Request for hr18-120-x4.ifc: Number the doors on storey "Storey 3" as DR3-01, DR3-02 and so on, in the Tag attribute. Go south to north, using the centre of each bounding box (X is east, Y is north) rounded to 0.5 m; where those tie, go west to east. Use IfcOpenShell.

First a look at what the model holds.

```python
import ifcopenshell
import ifcopenshell.util.element
import ifcopenshell.util.placement

model = ifcopenshell.open("hr18-120-x4.ifc")
print(model.schema)
storey = next(s for s in model.by_type("IfcBuildingStorey") if s.Name == "Storey 3")
doors = [e for e in ifcopenshell.util.element.get_decomposition(storey) if e.is_a("IfcDoor")]
for e in sorted(doors, key=lambda e: e.id()):
    origin = ifcopenshell.util.placement.get_local_placement(e.ObjectPlacement)[:3, 3]
    print(e.id(), e.Tag, e.Name, origin.round(2) + 0.0, sep=" | ")
```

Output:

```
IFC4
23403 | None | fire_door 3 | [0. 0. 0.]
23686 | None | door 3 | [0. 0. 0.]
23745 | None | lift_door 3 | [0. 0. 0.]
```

```python
import ifcopenshell
import ifcopenshell.geom
import ifcopenshell.util.element
import ifcopenshell.util.shape

model = ifcopenshell.open("hr18-120-x4.ifc")
settings = ifcopenshell.geom.settings()
settings.set("use-world-coords", True)


def centre(element):
    shape = ifcopenshell.geom.create_shape(settings, element)
    return ifcopenshell.util.shape.get_bbox_centroid(shape.geometry)


storey = next(s for s in model.by_type("IfcBuildingStorey") if s.Name == "Storey 3")
doors = [e for e in ifcopenshell.util.element.get_decomposition(storey) if e.is_a("IfcDoor")]

# Insertion points can sit at a corner or the storey origin, so sort by the geometry (in metres).
centres = {e: centre(e) for e in doors}
doors.sort(key=lambda e: (round(centres[e][1] / 0.5), centres[e][0]))

for i, e in enumerate(doors, start=1):
    number = f"DR3-{i:02d}"
    e.Tag = number
    print(e.id(), number)

model.write("hr18-120-x4_edited.ifc")
```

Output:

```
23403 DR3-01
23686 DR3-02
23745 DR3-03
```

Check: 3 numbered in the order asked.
